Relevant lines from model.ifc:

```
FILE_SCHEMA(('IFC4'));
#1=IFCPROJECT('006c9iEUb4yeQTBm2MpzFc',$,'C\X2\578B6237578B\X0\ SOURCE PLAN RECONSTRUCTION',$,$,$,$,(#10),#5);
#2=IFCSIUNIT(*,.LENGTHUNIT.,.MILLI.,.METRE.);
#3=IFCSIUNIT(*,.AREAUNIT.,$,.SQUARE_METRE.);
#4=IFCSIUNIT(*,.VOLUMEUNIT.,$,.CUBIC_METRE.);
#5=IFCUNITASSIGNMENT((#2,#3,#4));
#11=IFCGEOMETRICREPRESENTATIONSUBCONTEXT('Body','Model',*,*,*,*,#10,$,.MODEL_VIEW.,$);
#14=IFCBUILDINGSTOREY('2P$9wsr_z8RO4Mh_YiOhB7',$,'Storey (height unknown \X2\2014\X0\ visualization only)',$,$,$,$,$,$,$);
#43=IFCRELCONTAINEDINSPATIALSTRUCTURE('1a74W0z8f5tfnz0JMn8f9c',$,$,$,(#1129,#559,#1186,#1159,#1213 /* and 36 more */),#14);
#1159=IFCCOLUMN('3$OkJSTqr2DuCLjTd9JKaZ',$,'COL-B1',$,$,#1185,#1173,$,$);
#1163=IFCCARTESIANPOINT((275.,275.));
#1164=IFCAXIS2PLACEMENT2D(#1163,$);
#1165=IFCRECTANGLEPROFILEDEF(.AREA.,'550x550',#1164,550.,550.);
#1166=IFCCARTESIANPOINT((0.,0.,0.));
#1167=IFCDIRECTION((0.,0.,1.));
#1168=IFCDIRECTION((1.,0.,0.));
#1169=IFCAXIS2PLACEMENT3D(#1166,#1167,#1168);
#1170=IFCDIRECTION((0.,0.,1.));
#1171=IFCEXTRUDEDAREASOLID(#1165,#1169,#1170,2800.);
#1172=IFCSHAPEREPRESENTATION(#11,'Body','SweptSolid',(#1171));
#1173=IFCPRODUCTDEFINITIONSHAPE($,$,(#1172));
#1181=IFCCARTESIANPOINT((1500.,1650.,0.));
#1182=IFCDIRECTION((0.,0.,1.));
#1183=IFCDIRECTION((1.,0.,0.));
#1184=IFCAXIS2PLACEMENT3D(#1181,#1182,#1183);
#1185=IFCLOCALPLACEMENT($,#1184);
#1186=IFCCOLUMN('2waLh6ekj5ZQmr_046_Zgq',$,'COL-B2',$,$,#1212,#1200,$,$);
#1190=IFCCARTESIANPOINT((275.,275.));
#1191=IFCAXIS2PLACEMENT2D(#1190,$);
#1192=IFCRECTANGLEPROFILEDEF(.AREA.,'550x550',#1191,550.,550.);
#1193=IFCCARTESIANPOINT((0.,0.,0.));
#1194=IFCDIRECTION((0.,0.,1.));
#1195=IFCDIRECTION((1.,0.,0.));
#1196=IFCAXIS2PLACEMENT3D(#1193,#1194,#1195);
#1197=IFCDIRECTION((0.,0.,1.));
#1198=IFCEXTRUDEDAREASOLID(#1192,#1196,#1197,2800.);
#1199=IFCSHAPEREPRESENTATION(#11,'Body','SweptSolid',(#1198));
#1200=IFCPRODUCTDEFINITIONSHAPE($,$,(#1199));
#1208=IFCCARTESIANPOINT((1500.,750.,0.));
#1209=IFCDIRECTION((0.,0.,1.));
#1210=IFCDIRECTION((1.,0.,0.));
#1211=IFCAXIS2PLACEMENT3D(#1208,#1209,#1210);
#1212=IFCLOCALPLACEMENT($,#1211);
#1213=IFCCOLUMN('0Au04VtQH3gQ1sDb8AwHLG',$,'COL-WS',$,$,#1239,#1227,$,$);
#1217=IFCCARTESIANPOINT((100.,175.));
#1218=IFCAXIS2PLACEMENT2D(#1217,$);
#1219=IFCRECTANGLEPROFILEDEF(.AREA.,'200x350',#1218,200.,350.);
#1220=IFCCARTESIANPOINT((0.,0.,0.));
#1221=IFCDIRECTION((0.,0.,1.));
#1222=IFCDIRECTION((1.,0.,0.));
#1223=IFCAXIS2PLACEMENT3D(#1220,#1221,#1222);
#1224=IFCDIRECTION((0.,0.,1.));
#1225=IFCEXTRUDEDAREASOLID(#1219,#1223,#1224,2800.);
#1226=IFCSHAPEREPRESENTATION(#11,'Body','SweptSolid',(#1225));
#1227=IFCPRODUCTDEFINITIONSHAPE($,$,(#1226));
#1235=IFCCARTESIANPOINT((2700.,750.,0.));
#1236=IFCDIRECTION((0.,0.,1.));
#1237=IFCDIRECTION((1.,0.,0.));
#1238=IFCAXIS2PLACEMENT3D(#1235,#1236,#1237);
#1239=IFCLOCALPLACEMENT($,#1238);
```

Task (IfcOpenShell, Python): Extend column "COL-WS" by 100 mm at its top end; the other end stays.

```python
import ifcopenshell
import ifcopenshell.util.representation
import ifcopenshell.util.unit

model = ifcopenshell.open("model.ifc")
unit_scale = ifcopenshell.util.unit.calculate_unit_scale(model)

member = model.by_id(1213)
change = 0.1 / unit_scale

# The extrusion runs towards the end named, so only its depth changes.
body = ifcopenshell.util.representation.get_representation(member, "Model", "Body")
solid = body.Items[0]
old_length = solid.Depth
solid.Depth += change

print(f"length {old_length:g} -> {solid.Depth:g}")

model.write("model_edited.ifc")
```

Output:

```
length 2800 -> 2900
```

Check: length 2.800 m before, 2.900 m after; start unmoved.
